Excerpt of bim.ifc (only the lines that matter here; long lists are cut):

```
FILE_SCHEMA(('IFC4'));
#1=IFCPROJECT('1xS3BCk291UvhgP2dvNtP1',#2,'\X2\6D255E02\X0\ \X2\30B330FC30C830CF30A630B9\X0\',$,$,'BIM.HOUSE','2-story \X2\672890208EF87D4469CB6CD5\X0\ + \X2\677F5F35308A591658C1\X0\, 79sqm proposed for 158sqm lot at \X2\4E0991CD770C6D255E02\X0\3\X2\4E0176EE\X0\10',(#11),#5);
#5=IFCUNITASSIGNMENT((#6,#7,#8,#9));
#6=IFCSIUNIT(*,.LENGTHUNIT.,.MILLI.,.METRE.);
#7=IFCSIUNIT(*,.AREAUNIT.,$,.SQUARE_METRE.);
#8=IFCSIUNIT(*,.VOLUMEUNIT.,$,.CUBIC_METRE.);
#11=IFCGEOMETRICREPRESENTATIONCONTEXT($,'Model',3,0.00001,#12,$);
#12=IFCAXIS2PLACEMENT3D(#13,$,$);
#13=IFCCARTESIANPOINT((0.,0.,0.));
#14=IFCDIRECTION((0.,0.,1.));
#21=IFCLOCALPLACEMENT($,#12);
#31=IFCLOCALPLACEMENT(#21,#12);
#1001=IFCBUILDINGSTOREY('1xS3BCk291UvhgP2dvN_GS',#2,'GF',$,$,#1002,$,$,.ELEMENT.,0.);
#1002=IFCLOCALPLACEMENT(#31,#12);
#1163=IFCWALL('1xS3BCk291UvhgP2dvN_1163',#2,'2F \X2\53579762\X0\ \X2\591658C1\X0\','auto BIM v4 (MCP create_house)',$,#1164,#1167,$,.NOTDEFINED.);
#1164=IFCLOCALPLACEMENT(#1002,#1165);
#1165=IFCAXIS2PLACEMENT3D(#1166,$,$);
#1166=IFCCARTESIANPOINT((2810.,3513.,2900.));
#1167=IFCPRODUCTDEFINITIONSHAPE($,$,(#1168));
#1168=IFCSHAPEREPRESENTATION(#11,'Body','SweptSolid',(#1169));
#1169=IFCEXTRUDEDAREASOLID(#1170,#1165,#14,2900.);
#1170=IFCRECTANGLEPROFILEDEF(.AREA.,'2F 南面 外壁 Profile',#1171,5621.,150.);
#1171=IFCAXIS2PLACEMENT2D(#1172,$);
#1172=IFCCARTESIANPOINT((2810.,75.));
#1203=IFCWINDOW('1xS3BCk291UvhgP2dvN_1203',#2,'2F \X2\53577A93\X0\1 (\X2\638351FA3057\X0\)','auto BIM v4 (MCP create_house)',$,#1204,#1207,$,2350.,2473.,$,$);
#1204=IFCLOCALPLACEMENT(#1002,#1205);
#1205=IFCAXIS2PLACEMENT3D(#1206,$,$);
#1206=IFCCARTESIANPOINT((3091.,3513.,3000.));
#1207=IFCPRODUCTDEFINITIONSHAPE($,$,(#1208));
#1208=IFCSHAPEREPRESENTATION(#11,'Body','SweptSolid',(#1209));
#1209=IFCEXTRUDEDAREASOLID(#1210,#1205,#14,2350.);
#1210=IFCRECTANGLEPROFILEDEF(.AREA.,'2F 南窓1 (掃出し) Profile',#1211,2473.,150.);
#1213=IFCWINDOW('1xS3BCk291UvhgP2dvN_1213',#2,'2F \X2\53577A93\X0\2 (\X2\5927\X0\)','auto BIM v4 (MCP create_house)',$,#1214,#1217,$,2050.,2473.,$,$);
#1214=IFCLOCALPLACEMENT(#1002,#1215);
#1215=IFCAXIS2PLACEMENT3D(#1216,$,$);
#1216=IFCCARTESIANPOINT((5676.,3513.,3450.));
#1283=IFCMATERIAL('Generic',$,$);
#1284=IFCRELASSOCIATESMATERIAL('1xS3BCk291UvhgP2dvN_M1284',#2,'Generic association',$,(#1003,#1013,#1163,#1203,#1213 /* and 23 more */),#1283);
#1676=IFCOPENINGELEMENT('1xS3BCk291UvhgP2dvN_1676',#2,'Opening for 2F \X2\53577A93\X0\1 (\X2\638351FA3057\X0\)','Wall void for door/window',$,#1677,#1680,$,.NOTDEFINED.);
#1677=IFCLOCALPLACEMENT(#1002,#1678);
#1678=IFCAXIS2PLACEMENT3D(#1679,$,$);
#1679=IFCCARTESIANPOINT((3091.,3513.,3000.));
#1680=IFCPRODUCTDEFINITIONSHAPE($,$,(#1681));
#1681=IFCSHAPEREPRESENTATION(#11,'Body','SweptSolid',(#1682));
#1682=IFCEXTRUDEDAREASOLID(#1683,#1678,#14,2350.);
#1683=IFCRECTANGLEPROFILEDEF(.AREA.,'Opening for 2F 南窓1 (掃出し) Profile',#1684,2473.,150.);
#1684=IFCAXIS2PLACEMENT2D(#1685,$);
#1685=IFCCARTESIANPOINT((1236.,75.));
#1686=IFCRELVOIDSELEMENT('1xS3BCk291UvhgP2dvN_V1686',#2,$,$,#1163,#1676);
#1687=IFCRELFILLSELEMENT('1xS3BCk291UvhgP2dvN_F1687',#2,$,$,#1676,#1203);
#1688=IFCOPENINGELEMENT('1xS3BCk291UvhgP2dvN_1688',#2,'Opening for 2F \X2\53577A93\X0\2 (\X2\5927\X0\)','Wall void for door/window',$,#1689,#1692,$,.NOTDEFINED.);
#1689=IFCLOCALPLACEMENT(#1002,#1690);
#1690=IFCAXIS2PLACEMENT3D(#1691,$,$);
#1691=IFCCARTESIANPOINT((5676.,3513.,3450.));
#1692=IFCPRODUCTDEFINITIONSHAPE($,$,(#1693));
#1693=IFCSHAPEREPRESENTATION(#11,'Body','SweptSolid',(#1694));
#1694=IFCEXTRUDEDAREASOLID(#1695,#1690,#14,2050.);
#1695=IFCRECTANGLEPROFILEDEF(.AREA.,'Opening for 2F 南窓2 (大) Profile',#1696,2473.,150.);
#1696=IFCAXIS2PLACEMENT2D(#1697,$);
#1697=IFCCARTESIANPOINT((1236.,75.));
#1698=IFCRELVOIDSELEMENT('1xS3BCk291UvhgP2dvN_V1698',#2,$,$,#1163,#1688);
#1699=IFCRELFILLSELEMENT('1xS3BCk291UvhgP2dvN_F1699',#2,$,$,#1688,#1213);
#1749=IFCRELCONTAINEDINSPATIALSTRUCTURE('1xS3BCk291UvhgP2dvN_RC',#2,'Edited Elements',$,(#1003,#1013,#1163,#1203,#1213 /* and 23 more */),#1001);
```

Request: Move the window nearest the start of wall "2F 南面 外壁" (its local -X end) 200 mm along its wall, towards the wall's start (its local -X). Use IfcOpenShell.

```python
import ifcopenshell
import ifcopenshell.api.geometry
import ifcopenshell.util.placement

model = ifcopenshell.open("bim.ifc")

window = model.by_guid("1xS3BCk291UvhgP2dvN_1203")
opening = window.FillsVoids[0].RelatingOpeningElement
wall = opening.VoidsElements[0].RelatingBuildingElement

wall_matrix = ifcopenshell.util.placement.get_local_placement(wall.ObjectPlacement)
shift = wall_matrix[:3, 0] * -200.0
before = ifcopenshell.util.placement.get_local_placement(window.ObjectPlacement)[:3, 3].copy()

# The window is not placed relative to its opening, so move both.
for product in (opening, window):
    matrix = ifcopenshell.util.placement.get_local_placement(product.ObjectPlacement)
    matrix[:3, 3] += shift
    ifcopenshell.api.geometry.edit_object_placement(model, product=product, matrix=matrix, is_si=False)

after = ifcopenshell.util.placement.get_local_placement(window.ObjectPlacement)[:3, 3]
print("window moved by", (after - before).round(3) + 0.0)

model.write("bim_edited.ifc")
```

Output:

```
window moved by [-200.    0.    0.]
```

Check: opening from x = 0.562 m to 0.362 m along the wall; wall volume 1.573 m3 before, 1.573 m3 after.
